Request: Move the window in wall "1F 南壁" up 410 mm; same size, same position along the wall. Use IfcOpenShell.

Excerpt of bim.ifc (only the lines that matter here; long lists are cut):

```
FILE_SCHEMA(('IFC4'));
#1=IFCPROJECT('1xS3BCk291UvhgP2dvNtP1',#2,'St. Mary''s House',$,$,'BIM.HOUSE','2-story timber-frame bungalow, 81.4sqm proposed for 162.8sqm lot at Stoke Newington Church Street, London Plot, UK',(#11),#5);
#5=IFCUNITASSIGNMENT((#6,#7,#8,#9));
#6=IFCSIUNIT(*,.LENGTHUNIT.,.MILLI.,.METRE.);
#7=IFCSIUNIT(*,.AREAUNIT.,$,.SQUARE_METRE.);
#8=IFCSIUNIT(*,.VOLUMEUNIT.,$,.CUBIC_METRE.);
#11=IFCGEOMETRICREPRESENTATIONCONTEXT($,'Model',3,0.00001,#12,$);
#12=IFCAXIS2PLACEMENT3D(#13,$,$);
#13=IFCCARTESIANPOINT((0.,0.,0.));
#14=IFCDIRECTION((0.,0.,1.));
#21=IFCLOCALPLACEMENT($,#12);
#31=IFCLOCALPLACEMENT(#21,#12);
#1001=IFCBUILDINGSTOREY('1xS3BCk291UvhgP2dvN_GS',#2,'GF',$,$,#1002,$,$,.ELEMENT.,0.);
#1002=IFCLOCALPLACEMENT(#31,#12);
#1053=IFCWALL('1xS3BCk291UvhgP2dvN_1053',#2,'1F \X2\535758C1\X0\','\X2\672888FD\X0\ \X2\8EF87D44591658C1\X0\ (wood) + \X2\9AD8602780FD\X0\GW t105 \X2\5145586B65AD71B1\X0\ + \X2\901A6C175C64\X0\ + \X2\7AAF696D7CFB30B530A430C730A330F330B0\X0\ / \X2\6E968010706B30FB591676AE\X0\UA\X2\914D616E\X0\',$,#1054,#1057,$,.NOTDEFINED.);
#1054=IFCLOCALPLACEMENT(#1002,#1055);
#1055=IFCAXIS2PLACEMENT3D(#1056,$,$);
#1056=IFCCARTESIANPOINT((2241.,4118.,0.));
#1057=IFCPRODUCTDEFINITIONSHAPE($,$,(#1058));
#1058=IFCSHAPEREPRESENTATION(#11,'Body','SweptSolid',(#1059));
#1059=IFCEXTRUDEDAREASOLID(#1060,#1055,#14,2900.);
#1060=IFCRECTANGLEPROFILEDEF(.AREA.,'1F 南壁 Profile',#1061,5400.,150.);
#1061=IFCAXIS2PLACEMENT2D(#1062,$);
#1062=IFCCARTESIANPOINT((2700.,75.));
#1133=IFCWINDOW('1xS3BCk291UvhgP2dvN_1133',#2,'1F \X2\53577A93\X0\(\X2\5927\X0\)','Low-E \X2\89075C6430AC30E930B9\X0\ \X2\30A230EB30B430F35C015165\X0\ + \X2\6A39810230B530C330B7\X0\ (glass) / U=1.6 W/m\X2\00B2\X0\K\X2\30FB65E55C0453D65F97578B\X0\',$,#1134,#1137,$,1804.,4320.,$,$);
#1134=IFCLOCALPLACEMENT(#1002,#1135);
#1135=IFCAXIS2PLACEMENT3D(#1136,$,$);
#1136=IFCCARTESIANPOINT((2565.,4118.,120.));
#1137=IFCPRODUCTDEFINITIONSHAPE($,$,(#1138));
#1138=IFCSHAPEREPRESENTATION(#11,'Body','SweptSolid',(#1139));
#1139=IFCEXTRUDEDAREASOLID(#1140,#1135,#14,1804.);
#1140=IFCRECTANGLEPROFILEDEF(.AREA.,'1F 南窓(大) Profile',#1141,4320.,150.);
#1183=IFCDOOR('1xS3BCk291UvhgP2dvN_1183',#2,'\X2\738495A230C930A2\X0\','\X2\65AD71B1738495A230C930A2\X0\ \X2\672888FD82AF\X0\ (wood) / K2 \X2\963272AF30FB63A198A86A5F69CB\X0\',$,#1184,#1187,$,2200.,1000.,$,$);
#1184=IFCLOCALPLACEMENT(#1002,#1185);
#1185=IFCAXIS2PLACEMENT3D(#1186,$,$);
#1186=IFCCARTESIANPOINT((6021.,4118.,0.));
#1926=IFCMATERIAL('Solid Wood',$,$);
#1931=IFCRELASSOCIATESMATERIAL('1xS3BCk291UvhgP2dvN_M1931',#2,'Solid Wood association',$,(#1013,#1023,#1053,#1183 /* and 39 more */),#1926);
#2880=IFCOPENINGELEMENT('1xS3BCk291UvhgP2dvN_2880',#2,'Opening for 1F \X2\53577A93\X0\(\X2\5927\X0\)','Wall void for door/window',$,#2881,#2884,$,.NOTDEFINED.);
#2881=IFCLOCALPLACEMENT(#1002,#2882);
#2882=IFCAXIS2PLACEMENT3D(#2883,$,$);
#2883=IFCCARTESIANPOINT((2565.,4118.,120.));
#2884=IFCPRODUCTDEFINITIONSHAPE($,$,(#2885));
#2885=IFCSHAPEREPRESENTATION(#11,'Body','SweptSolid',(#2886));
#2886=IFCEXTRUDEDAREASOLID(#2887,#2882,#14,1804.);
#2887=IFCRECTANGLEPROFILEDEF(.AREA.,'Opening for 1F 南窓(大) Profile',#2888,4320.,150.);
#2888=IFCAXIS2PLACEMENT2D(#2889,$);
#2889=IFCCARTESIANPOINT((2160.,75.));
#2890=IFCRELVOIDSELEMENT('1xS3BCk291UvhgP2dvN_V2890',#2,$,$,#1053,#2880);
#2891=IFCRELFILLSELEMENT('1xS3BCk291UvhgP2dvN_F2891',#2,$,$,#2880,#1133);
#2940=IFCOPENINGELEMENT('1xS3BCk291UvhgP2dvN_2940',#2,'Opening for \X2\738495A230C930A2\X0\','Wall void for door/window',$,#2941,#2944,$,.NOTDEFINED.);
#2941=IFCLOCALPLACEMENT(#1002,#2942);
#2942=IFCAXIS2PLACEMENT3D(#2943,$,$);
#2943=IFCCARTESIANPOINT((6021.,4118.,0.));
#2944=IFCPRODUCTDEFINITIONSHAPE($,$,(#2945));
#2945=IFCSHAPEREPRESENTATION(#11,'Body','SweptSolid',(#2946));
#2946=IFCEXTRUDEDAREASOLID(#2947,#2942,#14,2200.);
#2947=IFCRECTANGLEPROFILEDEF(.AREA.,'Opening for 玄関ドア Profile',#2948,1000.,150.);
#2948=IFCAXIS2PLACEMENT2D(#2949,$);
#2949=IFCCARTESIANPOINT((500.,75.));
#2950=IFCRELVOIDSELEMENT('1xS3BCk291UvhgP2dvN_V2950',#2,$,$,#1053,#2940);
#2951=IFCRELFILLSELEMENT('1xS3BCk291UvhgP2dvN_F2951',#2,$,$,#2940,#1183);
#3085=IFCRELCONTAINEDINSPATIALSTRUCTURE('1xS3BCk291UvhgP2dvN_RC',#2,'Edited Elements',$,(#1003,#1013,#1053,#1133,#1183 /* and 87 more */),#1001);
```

```python
import numpy as np
import ifcopenshell
import ifcopenshell.api.geometry
import ifcopenshell.util.placement
import ifcopenshell.util.unit

model = ifcopenshell.open("bim.ifc")
unit_scale = ifcopenshell.util.unit.calculate_unit_scale(model)

window = model.by_id(1133)
opening = window.FillsVoids[0].RelatingOpeningElement
dz = 410.0

shift = np.array([0.0, 0.0, dz])
# The window is not placed relative to its opening, so move both.
for product in (opening, window):
    matrix = ifcopenshell.util.placement.get_local_placement(product.ObjectPlacement)
    matrix[:3, 3] += shift
    ifcopenshell.api.geometry.edit_object_placement(model, product=product, matrix=matrix, is_si=False)

print(f"moved by {dz * unit_scale:+.3f} m")

model.write("bim_v2.ifc")
```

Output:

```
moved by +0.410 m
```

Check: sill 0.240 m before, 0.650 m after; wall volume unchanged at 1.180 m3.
